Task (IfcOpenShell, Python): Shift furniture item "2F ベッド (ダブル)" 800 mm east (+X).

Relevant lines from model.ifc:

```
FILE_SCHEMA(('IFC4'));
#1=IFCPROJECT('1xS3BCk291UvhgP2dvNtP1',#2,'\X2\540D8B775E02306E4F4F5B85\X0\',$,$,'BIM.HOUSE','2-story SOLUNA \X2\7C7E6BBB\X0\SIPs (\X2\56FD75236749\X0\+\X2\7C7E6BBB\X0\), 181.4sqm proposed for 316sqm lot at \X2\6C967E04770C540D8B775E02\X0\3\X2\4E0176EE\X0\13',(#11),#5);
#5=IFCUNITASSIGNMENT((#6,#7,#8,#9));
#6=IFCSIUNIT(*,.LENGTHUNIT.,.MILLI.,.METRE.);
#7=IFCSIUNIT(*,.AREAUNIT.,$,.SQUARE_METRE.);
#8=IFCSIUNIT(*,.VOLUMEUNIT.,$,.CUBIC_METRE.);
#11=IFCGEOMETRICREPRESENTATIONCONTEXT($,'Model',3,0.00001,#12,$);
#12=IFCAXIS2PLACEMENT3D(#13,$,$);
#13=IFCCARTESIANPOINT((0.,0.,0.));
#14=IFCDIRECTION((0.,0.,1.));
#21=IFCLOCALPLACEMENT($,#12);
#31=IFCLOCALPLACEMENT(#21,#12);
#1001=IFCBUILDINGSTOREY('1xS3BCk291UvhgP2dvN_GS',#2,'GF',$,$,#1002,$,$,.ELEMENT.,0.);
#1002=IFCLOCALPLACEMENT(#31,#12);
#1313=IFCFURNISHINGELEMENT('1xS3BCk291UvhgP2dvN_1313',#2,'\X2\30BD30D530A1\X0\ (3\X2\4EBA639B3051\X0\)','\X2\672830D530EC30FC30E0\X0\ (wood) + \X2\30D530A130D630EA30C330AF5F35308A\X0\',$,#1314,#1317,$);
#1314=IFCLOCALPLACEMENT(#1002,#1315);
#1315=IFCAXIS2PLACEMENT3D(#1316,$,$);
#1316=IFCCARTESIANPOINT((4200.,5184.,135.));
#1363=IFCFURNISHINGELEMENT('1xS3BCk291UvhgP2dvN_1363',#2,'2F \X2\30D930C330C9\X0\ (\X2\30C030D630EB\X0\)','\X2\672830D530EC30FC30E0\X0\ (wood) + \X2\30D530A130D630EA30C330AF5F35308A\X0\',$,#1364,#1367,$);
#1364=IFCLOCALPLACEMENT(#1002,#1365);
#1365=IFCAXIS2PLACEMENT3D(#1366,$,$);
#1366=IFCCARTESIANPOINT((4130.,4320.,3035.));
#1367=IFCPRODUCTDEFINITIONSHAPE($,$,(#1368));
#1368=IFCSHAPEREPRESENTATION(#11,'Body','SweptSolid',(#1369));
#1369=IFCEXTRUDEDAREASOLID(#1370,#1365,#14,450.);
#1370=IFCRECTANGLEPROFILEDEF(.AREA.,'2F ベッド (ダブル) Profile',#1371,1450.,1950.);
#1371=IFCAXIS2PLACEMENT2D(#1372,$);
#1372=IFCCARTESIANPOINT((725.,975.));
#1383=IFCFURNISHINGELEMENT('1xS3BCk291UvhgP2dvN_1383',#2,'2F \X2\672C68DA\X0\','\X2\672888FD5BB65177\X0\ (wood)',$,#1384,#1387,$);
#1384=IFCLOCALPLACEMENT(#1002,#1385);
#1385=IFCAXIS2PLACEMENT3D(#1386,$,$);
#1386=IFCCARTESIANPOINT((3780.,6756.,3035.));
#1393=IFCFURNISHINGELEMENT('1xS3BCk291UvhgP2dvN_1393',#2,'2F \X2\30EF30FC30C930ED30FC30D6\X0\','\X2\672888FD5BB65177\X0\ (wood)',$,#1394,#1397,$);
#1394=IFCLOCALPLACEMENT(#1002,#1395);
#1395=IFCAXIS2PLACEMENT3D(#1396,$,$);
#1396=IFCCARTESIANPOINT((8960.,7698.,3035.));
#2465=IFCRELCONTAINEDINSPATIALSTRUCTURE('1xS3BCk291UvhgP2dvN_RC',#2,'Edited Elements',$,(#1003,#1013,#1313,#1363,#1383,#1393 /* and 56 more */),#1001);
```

```python
import ifcopenshell
import ifcopenshell.api.geometry
import ifcopenshell.util.placement
import ifcopenshell.util.unit

model = ifcopenshell.open("model.ifc")
unit_scale = ifcopenshell.util.unit.calculate_unit_scale(model)

item = model.by_guid("1xS3BCk291UvhgP2dvN_1363")
matrix = ifcopenshell.util.placement.get_local_placement(item.ObjectPlacement)
matrix[0, 3] += 0.8 / unit_scale
ifcopenshell.api.geometry.edit_object_placement(model, product=item, matrix=matrix, is_si=False)

print(ifcopenshell.util.placement.get_local_placement(item.ObjectPlacement).round(3) + 0.0)

model.write("model-out.ifc")
```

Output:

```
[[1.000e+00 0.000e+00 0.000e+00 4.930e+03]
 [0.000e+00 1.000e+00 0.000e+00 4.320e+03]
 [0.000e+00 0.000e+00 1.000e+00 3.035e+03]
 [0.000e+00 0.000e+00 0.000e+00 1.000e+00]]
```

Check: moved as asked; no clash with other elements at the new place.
